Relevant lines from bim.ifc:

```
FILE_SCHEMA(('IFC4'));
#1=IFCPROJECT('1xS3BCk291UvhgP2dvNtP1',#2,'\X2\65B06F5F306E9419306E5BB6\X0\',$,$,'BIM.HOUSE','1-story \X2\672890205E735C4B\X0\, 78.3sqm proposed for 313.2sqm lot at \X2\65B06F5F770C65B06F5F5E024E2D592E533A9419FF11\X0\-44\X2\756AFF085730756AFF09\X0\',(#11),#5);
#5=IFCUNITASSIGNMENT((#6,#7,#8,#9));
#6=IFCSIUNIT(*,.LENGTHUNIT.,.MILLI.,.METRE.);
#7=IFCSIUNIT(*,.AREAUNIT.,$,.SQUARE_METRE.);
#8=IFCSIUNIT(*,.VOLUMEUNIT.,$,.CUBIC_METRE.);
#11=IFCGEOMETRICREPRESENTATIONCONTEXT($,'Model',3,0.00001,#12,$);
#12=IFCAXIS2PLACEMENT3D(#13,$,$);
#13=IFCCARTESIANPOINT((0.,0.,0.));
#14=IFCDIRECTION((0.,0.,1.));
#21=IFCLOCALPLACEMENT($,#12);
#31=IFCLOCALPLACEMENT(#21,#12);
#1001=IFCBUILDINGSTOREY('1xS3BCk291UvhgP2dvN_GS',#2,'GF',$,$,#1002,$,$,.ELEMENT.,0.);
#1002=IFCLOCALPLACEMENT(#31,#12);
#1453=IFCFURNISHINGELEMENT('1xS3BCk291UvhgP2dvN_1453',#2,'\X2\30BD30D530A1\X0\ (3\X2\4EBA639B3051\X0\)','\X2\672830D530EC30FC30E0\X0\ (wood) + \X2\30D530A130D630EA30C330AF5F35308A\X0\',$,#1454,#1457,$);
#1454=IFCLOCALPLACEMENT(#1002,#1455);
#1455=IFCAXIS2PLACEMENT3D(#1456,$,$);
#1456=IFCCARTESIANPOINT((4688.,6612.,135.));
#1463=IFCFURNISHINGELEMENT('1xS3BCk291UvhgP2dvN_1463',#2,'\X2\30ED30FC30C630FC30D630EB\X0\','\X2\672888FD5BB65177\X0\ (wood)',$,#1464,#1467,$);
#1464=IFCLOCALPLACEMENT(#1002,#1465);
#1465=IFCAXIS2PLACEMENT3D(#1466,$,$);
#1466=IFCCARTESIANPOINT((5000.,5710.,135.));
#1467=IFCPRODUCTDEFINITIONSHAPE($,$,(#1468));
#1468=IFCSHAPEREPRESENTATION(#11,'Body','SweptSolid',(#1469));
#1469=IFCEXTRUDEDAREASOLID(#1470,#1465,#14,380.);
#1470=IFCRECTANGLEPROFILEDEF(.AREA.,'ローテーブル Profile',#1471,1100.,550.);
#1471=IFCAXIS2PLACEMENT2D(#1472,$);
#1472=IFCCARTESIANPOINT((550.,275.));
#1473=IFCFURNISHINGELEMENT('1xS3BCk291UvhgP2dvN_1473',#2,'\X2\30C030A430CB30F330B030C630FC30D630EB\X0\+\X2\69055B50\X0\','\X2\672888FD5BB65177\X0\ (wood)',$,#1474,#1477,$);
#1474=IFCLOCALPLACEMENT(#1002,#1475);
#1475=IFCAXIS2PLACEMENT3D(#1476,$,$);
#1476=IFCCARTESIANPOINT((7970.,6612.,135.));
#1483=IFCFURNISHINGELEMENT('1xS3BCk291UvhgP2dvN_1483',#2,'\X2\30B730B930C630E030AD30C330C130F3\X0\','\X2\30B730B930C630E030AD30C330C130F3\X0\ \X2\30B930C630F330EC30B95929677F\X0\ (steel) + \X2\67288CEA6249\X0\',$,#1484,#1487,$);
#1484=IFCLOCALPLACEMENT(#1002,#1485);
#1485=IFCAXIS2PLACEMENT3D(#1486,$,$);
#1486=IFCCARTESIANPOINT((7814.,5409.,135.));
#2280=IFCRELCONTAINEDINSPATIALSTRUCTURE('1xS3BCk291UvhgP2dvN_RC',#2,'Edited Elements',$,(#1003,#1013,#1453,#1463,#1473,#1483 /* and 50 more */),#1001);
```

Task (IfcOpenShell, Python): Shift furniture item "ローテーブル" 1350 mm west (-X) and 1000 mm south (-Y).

```python
import ifcopenshell
import ifcopenshell.api.geometry
import ifcopenshell.util.placement
import ifcopenshell.util.unit

model = ifcopenshell.open("bim.ifc")
unit_scale = ifcopenshell.util.unit.calculate_unit_scale(model)

item = model.by_guid("1xS3BCk291UvhgP2dvN_1463")
matrix = ifcopenshell.util.placement.get_local_placement(item.ObjectPlacement)
matrix[0, 3] -= 1.35 / unit_scale
matrix[1, 3] -= 1 / unit_scale
ifcopenshell.api.geometry.edit_object_placement(model, product=item, matrix=matrix, is_si=False)

print(ifcopenshell.util.placement.get_local_placement(item.ObjectPlacement).round(3) + 0.0)

model.write("bim_v2.ifc")
```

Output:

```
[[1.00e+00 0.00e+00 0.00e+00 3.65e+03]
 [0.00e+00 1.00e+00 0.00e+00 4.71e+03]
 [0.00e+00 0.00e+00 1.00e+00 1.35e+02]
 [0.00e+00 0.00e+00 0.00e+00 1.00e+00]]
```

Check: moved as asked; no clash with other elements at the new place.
